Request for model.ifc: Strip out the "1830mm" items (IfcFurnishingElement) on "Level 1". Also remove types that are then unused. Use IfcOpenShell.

First a look at what the model holds.

```python
import ifcopenshell
import ifcopenshell.util.element

model = ifcopenshell.open("model.ifc")
print(model.schema)
storey = next(s for s in model.by_type("IfcBuildingStorey") if s.Name == "Level 1")
furniture = [e for e in ifcopenshell.util.element.get_decomposition(storey) if e.is_a("IfcFurnishingElement")]
seen = {}
for e in furniture:
    element_type = ifcopenshell.util.element.get_type(e)
    name = element_type.Name if element_type not in (None, e) else None
    seen[name] = seen.get(name, 0) + 1
for name, count in sorted(seen.items(), key=str):
    print(count, "x", name)
```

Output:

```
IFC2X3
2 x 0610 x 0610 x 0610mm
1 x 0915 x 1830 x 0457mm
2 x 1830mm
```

```python
import ifcopenshell
import ifcopenshell.api.root
import ifcopenshell.util.element

model = ifcopenshell.open("model.ifc")

storey = next(s for s in model.by_type("IfcBuildingStorey") if s.Name == "Level 1")
furniture = [e for e in ifcopenshell.util.element.get_decomposition(storey) if e.is_a("IfcFurnishingElement")]
targets = [e for e in furniture if (t := ifcopenshell.util.element.get_type(e)) not in (None, e) and t.Name == "1830mm"]
types = {ifcopenshell.util.element.get_type(e) for e in targets} - {None, *targets}

for e in targets:
    ifcopenshell.api.root.remove_product(model, product=e)
print(len(targets), "removed")

unused = [t for t in types if not ifcopenshell.util.element.get_types(t)]
for t in unused:
    ifcopenshell.api.root.remove_product(model, product=t)
print(len(unused), "unused types removed")

model.write("model_updated.ifc")
```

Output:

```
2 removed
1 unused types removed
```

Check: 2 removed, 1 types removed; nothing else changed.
